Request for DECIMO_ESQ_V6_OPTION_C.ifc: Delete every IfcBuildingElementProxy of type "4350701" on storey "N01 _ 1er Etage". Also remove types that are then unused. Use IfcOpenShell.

First a look at what the model holds.

```python
import ifcopenshell
import ifcopenshell.util.element

model = ifcopenshell.open("DECIMO_ESQ_V6_OPTION_C.ifc")
print(model.schema)
storey = next(s for s in model.by_type("IfcBuildingStorey") if s.Name == "N01 _ 1er Etage")
proxies = [e for e in ifcopenshell.util.element.get_decomposition(storey) if e.is_a("IfcBuildingElementProxy")]
seen = {}
for e in proxies:
    element_type = ifcopenshell.util.element.get_type(e)
    name = element_type.Name if element_type not in (None, e) else None
    seen[name] = seen.get(name, 0) + 1
for name, count in sorted(seen.items(), key=str):
    print(count, "x", name)
```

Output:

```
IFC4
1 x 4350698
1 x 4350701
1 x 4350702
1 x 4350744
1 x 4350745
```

```python
import ifcopenshell
import ifcopenshell.api.root
import ifcopenshell.util.element

model = ifcopenshell.open("DECIMO_ESQ_V6_OPTION_C.ifc")

storey = next(s for s in model.by_type("IfcBuildingStorey") if s.Name == "N01 _ 1er Etage")
proxies = [e for e in ifcopenshell.util.element.get_decomposition(storey) if e.is_a("IfcBuildingElementProxy")]
targets = [e for e in proxies if (t := ifcopenshell.util.element.get_type(e)) not in (None, e) and t.Name == "4350701"]
types = {ifcopenshell.util.element.get_type(e) for e in targets} - {None, *targets}

for e in targets:
    ifcopenshell.api.root.remove_product(model, product=e)
print(len(targets), "removed")

unused = [t for t in types if not ifcopenshell.util.element.get_types(t)]
for t in unused:
    ifcopenshell.api.root.remove_product(model, product=t)
print(len(unused), "unused types removed")

model.write("DECIMO_ESQ_V6_OPTION_C_edited.ifc")
```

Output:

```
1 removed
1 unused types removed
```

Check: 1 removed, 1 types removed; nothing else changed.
